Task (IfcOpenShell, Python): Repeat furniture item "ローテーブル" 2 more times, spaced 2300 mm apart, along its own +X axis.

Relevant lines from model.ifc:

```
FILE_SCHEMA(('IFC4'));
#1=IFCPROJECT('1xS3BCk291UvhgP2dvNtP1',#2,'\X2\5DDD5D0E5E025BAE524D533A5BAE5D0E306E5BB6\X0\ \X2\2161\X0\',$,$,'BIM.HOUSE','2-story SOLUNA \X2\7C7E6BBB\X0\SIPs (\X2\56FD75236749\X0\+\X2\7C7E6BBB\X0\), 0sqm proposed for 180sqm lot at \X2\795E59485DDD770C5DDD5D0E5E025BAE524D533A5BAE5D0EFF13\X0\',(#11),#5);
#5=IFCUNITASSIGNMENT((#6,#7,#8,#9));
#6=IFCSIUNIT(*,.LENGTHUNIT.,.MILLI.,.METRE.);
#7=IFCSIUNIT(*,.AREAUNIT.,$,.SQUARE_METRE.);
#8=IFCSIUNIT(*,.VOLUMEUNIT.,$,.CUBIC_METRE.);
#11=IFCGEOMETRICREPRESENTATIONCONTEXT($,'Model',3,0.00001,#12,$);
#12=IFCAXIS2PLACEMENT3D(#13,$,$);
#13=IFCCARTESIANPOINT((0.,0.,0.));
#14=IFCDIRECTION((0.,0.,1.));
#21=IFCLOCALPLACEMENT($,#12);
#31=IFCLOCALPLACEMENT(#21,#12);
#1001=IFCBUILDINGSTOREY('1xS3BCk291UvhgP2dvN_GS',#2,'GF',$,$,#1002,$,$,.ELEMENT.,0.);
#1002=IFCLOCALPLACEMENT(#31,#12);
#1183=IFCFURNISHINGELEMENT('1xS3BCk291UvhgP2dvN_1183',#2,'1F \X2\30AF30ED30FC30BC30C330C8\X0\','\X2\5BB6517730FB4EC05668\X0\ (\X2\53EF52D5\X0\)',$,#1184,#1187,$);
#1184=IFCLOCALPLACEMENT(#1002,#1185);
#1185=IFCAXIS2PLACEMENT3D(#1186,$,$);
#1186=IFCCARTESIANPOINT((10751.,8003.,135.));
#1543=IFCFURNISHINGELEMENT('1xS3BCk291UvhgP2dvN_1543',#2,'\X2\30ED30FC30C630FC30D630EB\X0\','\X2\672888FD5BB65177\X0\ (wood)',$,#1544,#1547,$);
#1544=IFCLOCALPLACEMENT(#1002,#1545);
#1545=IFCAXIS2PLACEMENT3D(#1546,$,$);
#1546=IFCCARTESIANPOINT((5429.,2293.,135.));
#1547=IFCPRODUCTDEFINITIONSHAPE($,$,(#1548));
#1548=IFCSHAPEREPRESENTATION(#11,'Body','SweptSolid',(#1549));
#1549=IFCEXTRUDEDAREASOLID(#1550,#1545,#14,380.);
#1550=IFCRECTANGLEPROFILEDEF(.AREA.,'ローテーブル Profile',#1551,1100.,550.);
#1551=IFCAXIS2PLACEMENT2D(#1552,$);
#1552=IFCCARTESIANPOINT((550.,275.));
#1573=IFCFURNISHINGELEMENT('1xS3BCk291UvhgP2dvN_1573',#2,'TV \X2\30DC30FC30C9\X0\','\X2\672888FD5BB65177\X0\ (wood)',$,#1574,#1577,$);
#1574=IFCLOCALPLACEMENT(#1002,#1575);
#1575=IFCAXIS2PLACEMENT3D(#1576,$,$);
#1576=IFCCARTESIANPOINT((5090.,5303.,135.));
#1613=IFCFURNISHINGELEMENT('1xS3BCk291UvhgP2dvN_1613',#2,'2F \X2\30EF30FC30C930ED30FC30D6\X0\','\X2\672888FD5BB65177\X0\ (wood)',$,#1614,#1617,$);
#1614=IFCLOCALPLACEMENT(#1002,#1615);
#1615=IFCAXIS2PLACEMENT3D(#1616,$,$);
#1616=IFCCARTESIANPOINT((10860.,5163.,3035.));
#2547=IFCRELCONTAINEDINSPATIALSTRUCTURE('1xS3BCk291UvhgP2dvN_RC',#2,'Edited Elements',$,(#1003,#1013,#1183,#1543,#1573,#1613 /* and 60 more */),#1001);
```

```python
import ifcopenshell
import ifcopenshell.api.geometry
import ifcopenshell.api.root
import ifcopenshell.util.element
import ifcopenshell.util.placement
import ifcopenshell.util.unit

model = ifcopenshell.open("model.ifc")
unit_scale = ifcopenshell.util.unit.calculate_unit_scale(model)


def reuse_history(source, copy):
    """copy_class also copies each property set's owner history, people and application; keep the originals."""
    for rel in copy.IsDefinedBy:
        if rel.is_a("IfcRelDefinesByProperties") and (history := rel.RelatingPropertyDefinition.OwnerHistory):
            rel.RelatingPropertyDefinition.OwnerHistory = source.OwnerHistory
            ifcopenshell.util.element.remove_deep2(model, history)


source = model.by_guid("1xS3BCk291UvhgP2dvN_1543")
base = ifcopenshell.util.placement.get_local_placement(source.ObjectPlacement)
step = base[:3, 0] * 2.3 / unit_scale

for i in range(1, 3):
    copy = ifcopenshell.api.root.copy_class(model, product=source)
    copy.Representation = ifcopenshell.util.element.copy_deep(
        model, source.Representation, exclude=["IfcGeometricRepresentationContext", "IfcRepresentationMap"]
    )
    reuse_history(source, copy)
    matrix = base.copy()
    matrix[:3, 3] += i * step
    print("added at", matrix[:3, 3].round(3) + 0.0)
    ifcopenshell.api.geometry.edit_object_placement(model, product=copy, matrix=matrix, is_si=False)

model.write("model_v2.ifc")
```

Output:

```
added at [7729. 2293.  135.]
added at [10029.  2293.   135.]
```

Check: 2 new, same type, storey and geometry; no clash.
